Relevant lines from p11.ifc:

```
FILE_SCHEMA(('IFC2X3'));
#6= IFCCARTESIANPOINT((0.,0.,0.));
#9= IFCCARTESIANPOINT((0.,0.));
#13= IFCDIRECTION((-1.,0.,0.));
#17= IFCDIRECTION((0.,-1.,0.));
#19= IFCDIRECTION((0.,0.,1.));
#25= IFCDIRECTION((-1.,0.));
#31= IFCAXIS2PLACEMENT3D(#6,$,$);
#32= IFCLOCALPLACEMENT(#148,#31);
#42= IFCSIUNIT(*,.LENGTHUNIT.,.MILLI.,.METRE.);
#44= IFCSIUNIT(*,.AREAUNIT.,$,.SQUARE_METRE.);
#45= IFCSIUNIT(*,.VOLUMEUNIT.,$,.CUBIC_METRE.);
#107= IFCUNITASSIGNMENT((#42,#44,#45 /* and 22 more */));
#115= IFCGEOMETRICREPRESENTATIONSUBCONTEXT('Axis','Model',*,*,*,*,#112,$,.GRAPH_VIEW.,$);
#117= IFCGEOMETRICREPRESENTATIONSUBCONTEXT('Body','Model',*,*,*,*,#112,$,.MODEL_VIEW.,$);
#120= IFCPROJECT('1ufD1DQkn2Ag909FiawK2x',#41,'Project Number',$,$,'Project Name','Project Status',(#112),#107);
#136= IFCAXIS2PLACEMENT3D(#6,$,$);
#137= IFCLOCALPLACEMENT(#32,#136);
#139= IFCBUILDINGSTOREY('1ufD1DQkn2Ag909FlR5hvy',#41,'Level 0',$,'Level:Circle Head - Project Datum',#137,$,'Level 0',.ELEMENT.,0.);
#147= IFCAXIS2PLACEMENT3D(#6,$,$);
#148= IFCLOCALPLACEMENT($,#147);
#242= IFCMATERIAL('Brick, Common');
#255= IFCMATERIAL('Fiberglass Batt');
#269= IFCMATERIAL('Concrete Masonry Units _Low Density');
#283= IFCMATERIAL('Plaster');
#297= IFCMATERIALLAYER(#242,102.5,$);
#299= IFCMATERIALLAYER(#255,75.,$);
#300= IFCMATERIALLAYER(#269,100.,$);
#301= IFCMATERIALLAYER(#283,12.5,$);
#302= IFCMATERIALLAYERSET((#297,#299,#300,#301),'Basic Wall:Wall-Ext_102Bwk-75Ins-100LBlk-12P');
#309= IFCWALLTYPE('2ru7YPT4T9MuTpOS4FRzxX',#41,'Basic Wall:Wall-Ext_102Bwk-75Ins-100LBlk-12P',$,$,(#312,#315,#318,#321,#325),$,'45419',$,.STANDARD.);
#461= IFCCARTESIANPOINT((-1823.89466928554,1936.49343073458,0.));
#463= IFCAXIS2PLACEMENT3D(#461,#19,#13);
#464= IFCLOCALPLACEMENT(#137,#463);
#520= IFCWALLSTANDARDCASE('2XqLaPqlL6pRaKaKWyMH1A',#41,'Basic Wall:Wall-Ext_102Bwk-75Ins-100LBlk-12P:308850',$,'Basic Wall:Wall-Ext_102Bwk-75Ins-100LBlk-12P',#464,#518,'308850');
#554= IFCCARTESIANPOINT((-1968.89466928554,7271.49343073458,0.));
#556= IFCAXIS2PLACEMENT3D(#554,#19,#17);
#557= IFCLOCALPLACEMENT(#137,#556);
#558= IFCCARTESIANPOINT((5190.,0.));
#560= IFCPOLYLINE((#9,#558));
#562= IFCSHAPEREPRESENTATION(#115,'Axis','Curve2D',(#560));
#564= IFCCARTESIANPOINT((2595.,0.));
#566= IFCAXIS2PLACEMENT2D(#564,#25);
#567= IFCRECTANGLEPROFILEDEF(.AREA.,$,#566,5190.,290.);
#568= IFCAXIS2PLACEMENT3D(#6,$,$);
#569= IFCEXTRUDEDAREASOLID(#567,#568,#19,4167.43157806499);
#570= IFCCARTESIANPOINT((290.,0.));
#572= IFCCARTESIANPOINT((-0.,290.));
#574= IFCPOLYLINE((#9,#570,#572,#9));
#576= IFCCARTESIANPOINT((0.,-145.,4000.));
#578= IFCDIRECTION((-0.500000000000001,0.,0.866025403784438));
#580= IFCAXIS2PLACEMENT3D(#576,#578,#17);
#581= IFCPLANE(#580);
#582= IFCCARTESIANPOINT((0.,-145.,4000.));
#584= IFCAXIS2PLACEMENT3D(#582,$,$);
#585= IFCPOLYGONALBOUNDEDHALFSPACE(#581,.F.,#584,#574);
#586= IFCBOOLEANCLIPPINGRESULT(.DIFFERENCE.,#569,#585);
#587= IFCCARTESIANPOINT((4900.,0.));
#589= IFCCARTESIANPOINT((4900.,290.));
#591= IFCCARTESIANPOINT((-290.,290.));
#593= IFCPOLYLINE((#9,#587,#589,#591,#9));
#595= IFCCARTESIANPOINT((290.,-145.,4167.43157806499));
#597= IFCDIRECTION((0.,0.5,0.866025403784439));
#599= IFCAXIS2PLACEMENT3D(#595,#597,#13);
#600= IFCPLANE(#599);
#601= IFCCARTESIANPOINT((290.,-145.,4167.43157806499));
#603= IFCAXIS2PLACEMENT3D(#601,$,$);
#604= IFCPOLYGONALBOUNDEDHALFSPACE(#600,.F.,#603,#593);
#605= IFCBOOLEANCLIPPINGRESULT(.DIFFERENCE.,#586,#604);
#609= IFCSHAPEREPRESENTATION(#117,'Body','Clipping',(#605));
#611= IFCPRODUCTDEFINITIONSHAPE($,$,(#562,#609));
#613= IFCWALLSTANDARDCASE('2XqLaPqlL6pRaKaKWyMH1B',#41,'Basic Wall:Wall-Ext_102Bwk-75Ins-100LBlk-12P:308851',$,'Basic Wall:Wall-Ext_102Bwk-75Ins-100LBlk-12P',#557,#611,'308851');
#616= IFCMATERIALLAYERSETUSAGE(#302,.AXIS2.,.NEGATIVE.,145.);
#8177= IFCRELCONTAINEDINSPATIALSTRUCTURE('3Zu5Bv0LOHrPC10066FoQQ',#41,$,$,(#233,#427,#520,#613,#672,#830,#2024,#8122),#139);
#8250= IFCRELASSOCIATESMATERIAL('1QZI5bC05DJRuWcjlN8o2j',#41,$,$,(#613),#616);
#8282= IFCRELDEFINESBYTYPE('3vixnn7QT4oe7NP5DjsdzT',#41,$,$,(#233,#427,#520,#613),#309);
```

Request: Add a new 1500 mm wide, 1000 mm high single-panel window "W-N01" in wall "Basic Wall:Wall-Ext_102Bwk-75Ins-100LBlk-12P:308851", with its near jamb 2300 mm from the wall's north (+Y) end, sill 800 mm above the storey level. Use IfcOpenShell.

```python
import numpy as np
import ifcopenshell
import ifcopenshell.api.feature
import ifcopenshell.api.geometry
import ifcopenshell.api.root
import ifcopenshell.api.spatial
import ifcopenshell.api.type
import ifcopenshell.geom
import ifcopenshell.util.element
import ifcopenshell.util.placement
import ifcopenshell.util.representation
import ifcopenshell.util.shape
import ifcopenshell.util.unit

model = ifcopenshell.open("p11.ifc")
unit_scale = ifcopenshell.util.unit.calculate_unit_scale(model)
settings = ifcopenshell.geom.settings()


def volume(element):
    """Net volume in cubic metres, openings subtracted."""
    shape = ifcopenshell.geom.create_shape(settings, element)
    return ifcopenshell.util.shape.get_volume(shape.geometry)


wall = model.by_guid("2XqLaPqlL6pRaKaKWyMH1B")
storey = ifcopenshell.util.element.get_container(wall, ifc_class="IfcBuildingStorey")
context = ifcopenshell.util.representation.get_context(model, "Model", "Body", "MODEL_VIEW")
before = volume(wall)

width, height, from_end, sill = 1.5, 1, 2.3, 0.8  # metres

# The wall runs along its own X axis, and the end named is its -X end.
wall_shape = ifcopenshell.geom.create_shape(settings, wall)
x, y, z = ifcopenshell.util.shape.get_vertices(wall_shape.geometry).T
start = x.min() + from_end
face, thickness = float(y.min()), float(y.max() - y.min())
wall_matrix = ifcopenshell.util.placement.get_local_placement(wall.ObjectPlacement)
level = ifcopenshell.util.placement.get_local_placement(storey.ObjectPlacement)[2, 3]


def in_wall(x, y):
    """Placement at x, y metres in the wall's axes, at sill height."""
    matrix = wall_matrix.copy()
    matrix[:, 3] = wall_matrix @ np.array([x / unit_scale, y / unit_scale, 0.0, 1.0])
    matrix[2, 3] = level + sill / unit_scale
    return matrix


# Opening: a box that overshoots both wall faces by 50 mm.
opening = ifcopenshell.api.root.create_entity(model, ifc_class="IfcOpeningElement")
box = ifcopenshell.api.geometry.add_wall_representation(
    model, context=context, length=width, height=height, thickness=thickness + 0.1
)
ifcopenshell.api.geometry.assign_representation(model, product=opening, representation=box)
ifcopenshell.api.geometry.edit_object_placement(model, product=opening, matrix=in_wall(start, face - 0.05), is_si=False)
ifcopenshell.api.feature.add_feature(model, feature=opening, element=wall)

window = ifcopenshell.api.root.create_entity(model, ifc_class="IfcWindow", name="W-N01")
window.OverallWidth, window.OverallHeight = width / unit_scale, height / unit_scale
body = ifcopenshell.api.geometry.add_window_representation(
    model,
    context=context,
    overall_width=window.OverallWidth,
    overall_height=window.OverallHeight,
    partition_type="SINGLE_PANEL",
)
ifcopenshell.api.geometry.assign_representation(model, product=window, representation=body)
ifcopenshell.api.spatial.assign_container(model, products=[window], relating_structure=storey)
fills = ifcopenshell.api.feature.add_filling(model, opening=opening, element=window)
fills.OwnerHistory = window.OwnerHistory  # required in IFC2X3

# IFC2X3 keeps the operation on the window style.
style = ifcopenshell.api.root.create_entity(model, ifc_class="IfcWindowStyle", name="W-N01")
style.OperationType, style.ConstructionType = "SINGLE_PANEL", "NOTDEFINED"
style.ParameterTakesPrecedence = style.Sizeable = False
ifcopenshell.api.type.assign_type(model, related_objects=[window], relating_type=style)

# Centre the window in the wall's thickness.
ifcopenshell.api.geometry.edit_object_placement(model, product=window, matrix=in_wall(start, face), is_si=False)
window_shape = ifcopenshell.geom.create_shape(settings, window)
depth = ifcopenshell.util.shape.get_vertices(window_shape.geometry)[:, 1]
offset = face + thickness / 2 - (depth.min() + depth.max()) / 2
ifcopenshell.api.geometry.edit_object_placement(model, product=window, matrix=in_wall(start, offset), is_si=False)

after = volume(wall)

print(f"wall volume {before:.3f} -> {after:.3f} m3")

model.write("p11_v2.ifc")
```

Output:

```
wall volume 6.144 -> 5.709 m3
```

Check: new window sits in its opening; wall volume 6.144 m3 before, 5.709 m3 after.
